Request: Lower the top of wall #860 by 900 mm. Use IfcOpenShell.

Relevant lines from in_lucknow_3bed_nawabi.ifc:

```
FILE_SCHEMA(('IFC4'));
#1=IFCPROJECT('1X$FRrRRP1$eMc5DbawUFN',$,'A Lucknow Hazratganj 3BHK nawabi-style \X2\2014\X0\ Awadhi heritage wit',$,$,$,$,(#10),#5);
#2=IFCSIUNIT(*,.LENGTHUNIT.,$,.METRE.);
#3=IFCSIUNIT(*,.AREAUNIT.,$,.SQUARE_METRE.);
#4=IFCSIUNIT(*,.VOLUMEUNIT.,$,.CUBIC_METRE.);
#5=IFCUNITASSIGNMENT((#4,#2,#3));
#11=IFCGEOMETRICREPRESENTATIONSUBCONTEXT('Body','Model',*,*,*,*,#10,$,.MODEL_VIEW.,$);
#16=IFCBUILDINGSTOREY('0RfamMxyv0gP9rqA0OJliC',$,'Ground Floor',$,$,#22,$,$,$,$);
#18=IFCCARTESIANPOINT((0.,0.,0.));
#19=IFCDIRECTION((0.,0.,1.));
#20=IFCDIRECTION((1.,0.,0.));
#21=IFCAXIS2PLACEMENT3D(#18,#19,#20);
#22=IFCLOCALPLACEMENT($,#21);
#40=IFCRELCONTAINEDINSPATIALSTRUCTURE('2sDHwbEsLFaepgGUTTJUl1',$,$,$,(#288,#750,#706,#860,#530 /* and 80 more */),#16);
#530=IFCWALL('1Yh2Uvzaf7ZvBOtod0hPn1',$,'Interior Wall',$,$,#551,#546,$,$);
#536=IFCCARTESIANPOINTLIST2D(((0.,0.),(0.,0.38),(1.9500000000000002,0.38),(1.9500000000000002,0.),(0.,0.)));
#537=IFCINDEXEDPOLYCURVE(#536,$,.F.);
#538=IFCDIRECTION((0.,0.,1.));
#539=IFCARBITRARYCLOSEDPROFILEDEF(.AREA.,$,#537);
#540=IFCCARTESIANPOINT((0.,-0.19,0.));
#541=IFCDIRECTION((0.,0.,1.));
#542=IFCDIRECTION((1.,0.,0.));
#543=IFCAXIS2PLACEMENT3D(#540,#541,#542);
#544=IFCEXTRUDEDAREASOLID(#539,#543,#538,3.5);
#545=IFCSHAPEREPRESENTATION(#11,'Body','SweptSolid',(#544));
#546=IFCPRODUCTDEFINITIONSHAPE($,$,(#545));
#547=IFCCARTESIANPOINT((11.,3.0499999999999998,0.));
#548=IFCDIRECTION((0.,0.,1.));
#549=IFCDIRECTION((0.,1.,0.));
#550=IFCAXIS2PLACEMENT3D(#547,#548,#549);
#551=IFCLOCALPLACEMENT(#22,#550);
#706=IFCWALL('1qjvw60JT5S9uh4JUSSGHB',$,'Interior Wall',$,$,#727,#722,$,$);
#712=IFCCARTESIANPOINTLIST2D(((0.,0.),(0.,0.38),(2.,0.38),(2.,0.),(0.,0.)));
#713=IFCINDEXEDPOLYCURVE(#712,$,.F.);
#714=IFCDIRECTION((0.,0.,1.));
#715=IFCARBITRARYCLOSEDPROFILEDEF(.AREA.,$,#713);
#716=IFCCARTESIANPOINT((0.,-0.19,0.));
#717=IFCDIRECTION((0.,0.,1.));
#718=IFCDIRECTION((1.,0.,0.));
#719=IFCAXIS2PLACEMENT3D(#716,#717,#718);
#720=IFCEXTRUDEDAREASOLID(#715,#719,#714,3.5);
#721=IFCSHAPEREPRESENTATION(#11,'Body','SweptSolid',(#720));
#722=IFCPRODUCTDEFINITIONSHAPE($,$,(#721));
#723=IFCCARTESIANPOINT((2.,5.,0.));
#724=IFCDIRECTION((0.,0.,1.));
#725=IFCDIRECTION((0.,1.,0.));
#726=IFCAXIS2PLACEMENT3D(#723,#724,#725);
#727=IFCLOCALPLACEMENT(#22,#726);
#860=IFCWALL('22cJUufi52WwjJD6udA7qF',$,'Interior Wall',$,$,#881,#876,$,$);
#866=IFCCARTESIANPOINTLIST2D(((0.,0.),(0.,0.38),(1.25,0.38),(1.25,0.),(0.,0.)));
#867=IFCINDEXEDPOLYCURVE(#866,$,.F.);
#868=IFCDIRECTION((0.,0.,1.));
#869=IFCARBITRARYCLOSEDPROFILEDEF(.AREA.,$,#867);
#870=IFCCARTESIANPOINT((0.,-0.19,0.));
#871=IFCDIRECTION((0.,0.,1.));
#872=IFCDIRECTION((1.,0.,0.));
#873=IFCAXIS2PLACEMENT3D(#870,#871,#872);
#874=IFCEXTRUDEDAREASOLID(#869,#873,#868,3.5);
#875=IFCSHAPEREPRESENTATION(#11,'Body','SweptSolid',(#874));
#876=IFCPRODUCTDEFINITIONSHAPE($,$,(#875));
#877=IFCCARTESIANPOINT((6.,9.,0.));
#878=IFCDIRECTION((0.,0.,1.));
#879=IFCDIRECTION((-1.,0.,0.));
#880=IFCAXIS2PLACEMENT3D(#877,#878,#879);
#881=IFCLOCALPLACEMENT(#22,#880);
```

```python
import ifcopenshell
import ifcopenshell.geom
import ifcopenshell.util.representation
import ifcopenshell.util.shape

model = ifcopenshell.open("in_lucknow_3bed_nawabi.ifc")
settings = ifcopenshell.geom.settings()


def volume(element):
    """Net volume in cubic metres, openings subtracted."""
    shape = ifcopenshell.geom.create_shape(settings, element)
    return ifcopenshell.util.shape.get_volume(shape.geometry)


wall = model.by_guid("22cJUufi52WwjJD6udA7qF")
before = volume(wall)

body = ifcopenshell.util.representation.get_representation(wall, "Model", "Body")
solid = body.Items[0]
old_height = solid.Depth
solid.Depth -= 0.9
after = volume(wall)

print(f"height {old_height:g} -> {solid.Depth:g}, volume {before:.3f} -> {after:.3f} m3")

model.write("in_lucknow_3bed_nawabi-out.ifc")
```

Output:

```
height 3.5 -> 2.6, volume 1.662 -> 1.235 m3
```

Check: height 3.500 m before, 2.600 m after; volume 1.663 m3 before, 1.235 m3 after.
